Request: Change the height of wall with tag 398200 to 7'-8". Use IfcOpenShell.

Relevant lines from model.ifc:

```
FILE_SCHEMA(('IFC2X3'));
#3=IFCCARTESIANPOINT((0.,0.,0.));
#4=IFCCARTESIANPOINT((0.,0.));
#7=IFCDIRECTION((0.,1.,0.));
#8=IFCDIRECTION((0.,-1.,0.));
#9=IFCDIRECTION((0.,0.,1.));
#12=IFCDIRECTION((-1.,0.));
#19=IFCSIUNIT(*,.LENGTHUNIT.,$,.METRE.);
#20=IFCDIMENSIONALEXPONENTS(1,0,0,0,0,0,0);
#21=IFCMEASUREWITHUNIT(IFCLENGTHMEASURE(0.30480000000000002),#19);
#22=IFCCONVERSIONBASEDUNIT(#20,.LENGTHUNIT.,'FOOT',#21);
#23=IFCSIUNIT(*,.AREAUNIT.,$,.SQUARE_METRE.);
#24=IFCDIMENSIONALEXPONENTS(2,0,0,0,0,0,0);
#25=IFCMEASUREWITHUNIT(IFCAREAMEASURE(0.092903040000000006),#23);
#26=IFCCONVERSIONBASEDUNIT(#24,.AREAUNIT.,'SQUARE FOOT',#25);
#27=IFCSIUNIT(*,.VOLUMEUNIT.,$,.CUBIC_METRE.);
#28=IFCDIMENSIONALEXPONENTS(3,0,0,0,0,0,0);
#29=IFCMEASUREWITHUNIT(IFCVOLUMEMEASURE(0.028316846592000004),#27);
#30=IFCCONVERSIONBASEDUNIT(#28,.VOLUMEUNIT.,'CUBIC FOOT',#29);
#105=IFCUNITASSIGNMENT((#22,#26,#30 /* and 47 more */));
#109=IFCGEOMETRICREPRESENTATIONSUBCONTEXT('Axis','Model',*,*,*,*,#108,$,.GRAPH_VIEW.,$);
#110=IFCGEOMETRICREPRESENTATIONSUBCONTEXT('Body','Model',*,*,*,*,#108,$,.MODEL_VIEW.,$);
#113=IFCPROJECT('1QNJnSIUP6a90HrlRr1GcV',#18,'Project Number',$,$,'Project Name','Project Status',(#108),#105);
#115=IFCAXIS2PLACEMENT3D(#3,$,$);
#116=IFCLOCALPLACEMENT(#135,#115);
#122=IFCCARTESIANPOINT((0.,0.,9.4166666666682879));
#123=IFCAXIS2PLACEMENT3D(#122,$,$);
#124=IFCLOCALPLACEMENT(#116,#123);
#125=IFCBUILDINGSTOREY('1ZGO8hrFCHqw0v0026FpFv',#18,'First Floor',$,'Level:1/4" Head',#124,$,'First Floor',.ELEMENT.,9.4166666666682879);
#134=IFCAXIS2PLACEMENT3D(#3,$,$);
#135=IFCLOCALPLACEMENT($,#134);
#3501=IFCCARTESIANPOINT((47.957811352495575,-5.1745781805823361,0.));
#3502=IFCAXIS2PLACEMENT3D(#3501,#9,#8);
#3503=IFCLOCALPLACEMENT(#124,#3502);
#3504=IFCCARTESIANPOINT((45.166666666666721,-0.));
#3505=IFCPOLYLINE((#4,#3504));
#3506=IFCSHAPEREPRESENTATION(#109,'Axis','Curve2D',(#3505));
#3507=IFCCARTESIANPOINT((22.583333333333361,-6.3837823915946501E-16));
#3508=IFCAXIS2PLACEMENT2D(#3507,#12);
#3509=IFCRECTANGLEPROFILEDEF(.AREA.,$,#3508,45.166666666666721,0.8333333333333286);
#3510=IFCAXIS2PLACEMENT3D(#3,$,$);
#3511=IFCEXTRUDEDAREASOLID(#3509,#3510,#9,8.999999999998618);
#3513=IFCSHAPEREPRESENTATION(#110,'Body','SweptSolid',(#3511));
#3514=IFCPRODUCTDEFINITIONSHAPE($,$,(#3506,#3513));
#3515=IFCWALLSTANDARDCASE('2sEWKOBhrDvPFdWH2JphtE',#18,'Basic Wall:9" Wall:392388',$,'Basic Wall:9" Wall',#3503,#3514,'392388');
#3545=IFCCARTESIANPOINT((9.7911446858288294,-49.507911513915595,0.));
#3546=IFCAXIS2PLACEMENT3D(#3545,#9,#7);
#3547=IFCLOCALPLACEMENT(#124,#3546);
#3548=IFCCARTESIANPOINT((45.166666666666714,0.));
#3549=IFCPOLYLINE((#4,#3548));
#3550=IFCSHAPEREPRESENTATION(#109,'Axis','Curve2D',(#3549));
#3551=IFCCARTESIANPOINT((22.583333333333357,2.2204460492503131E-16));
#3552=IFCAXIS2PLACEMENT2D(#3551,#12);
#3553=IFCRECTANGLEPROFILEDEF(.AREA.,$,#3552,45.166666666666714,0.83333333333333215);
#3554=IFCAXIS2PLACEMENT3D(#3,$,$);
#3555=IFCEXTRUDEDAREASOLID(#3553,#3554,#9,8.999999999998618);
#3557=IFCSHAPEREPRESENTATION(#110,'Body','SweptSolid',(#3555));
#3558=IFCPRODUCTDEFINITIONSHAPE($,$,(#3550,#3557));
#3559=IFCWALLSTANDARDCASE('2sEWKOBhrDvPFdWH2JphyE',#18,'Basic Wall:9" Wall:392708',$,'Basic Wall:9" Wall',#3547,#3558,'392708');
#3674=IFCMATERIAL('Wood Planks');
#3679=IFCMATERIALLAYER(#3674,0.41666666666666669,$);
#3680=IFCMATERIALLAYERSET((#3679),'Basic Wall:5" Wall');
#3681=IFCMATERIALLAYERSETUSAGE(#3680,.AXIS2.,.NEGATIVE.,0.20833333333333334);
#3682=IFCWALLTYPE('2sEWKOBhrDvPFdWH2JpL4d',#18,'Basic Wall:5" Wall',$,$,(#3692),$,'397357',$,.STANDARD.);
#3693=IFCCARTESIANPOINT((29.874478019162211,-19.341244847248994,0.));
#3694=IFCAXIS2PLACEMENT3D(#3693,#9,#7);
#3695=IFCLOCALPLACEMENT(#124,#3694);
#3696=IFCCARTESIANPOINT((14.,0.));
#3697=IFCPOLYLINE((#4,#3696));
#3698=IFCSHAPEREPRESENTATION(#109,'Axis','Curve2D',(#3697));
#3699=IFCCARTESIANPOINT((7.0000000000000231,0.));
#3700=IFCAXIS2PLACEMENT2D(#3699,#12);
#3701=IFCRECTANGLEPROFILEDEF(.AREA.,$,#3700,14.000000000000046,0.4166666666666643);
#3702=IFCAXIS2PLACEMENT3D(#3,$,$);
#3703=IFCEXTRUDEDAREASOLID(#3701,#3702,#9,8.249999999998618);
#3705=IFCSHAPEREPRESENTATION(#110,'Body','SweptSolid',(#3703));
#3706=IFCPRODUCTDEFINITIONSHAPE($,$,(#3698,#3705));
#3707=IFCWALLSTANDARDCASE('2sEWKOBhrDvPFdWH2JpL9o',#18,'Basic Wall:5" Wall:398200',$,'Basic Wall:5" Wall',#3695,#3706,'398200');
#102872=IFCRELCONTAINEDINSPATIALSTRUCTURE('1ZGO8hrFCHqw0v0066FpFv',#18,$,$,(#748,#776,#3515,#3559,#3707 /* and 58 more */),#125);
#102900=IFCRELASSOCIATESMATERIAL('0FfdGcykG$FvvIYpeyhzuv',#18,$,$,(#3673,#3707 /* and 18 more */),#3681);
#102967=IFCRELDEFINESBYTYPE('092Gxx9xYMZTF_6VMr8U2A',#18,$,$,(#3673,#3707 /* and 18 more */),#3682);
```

```python
import ifcopenshell
import ifcopenshell.geom
import ifcopenshell.util.representation
import ifcopenshell.util.shape
import ifcopenshell.util.unit

model = ifcopenshell.open("model.ifc")
unit_scale = ifcopenshell.util.unit.calculate_unit_scale(model)
settings = ifcopenshell.geom.settings()


def volume(element):
    """Net volume in cubic metres, openings subtracted."""
    shape = ifcopenshell.geom.create_shape(settings, element)
    return ifcopenshell.util.shape.get_volume(shape.geometry)


wall = model.by_guid("2sEWKOBhrDvPFdWH2JpL9o")
before = volume(wall)

body = ifcopenshell.util.representation.get_representation(wall, "Model", "Body")
solid = body.Items[0]
old_height = solid.Depth
solid.Depth = 92 * 0.0254 / unit_scale
after = volume(wall)

print(f"height {old_height:g} -> {solid.Depth:g}, volume {before:.3f} -> {after:.3f} m3")

model.write("model_rev.ifc")
```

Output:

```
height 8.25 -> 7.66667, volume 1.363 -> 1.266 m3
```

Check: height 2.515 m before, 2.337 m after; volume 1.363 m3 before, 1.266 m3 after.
